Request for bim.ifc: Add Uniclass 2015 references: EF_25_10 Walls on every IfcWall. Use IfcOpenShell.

First a look at what the model holds.

```python
import ifcopenshell

model = ifcopenshell.open("bim.ifc")
print(model.schema)
print("classifications:", [c.Name for c in model.by_type("IfcClassification")])
for ifc_class in ("IfcDoor", "IfcRoof", "IfcStair", "IfcWall", "IfcWindow"):
    print(ifc_class, len(model.by_type(ifc_class)))
```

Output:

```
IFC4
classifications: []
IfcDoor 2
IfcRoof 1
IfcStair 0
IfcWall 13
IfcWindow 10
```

```python
import ifcopenshell
import ifcopenshell.api.classification

model = ifcopenshell.open("bim.ifc")

system = ifcopenshell.api.classification.add_classification(model, classification="Uniclass 2015")

codes = {
    "IfcWall": ("EF_25_10", "Walls"),
}
for ifc_class, (code, name) in codes.items():
    products = model.by_type(ifc_class)
    ifcopenshell.api.classification.add_reference(
        model, products=products, classification=system, identification=code, name=name
    )
    print(code, len(products))

model.write("bim_updated.ifc")
```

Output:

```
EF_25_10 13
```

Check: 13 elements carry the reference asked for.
